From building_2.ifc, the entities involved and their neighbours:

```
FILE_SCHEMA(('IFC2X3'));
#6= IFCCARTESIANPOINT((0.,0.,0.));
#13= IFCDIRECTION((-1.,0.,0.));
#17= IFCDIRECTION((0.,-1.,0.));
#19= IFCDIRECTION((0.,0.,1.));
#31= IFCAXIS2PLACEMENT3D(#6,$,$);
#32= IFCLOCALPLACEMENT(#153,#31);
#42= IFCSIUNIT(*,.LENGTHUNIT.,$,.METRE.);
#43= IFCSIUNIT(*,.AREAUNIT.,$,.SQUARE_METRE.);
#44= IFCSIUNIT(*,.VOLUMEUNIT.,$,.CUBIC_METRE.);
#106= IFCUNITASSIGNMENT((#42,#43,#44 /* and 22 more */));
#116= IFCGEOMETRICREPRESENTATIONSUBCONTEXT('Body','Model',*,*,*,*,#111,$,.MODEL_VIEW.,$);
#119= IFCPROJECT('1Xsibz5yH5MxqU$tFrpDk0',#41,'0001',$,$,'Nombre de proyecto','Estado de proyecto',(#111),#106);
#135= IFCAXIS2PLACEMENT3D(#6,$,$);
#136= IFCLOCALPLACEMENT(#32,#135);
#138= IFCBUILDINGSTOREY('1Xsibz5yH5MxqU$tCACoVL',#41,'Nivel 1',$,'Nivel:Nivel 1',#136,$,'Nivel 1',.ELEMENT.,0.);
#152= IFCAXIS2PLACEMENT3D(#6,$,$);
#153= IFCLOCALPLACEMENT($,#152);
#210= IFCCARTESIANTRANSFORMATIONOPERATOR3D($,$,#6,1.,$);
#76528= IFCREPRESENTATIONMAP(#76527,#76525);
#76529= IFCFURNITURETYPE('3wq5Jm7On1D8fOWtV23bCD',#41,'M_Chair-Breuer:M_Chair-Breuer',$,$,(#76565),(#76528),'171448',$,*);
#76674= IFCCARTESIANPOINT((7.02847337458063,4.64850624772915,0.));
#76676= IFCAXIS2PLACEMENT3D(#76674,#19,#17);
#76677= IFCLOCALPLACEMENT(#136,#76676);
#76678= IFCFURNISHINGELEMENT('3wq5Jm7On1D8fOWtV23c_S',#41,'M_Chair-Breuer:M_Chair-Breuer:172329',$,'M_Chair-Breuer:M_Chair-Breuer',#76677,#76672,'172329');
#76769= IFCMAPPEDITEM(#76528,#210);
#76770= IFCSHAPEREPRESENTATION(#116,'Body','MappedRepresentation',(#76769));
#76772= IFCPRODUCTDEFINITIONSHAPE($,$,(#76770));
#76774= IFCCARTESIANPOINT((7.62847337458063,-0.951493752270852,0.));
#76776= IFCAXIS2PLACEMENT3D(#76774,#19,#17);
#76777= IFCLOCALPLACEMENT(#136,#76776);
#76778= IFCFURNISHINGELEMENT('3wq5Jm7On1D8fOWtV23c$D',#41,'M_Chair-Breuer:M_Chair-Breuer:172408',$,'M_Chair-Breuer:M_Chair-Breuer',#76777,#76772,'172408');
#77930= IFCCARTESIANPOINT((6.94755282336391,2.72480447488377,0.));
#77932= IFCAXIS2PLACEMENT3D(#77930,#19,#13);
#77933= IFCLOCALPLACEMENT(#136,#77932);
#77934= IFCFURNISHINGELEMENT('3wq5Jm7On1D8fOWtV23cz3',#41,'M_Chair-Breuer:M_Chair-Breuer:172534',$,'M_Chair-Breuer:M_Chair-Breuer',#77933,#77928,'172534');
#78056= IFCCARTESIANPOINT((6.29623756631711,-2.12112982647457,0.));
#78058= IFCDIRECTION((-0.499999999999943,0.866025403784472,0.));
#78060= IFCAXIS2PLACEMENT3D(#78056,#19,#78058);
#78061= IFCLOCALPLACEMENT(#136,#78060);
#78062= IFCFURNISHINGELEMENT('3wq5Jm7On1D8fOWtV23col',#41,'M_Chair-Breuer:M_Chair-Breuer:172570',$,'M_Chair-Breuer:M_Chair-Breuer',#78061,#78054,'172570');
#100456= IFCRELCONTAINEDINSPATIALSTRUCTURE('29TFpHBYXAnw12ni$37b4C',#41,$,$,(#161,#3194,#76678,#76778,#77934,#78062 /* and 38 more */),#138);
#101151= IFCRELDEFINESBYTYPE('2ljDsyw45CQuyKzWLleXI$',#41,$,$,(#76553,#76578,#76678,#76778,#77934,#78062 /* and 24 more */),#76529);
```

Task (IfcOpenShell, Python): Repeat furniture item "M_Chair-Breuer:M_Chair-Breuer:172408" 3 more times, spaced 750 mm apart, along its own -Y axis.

```python
import ifcopenshell
import ifcopenshell.api.geometry
import ifcopenshell.api.root
import ifcopenshell.util.element
import ifcopenshell.util.placement
import ifcopenshell.util.unit

model = ifcopenshell.open("building_2.ifc")
unit_scale = ifcopenshell.util.unit.calculate_unit_scale(model)


def reuse_history(source, copy):
    """copy_class also copies each property set's owner history, people and application; keep the originals."""
    for rel in copy.IsDefinedBy:
        if rel.is_a("IfcRelDefinesByProperties") and (history := rel.RelatingPropertyDefinition.OwnerHistory):
            rel.RelatingPropertyDefinition.OwnerHistory = source.OwnerHistory
            ifcopenshell.util.element.remove_deep2(model, history)


source = model.by_guid("3wq5Jm7On1D8fOWtV23c$D")
base = ifcopenshell.util.placement.get_local_placement(source.ObjectPlacement)
step = -base[:3, 1] * 0.75 / unit_scale

for i in range(1, 4):
    copy = ifcopenshell.api.root.copy_class(model, product=source)
    copy.Representation = ifcopenshell.util.element.copy_deep(
        model, source.Representation, exclude=["IfcGeometricRepresentationContext", "IfcRepresentationMap"]
    )
    copy.Name = "M_Chair-Breuer:M_Chair-Breuer"
    copy.Tag = None
    reuse_history(source, copy)
    matrix = base.copy()
    matrix[:3, 3] += i * step
    print("added at", matrix[:3, 3].round(3) + 0.0)
    ifcopenshell.api.geometry.edit_object_placement(model, product=copy, matrix=matrix, is_si=False)

model.write("building_2_v2.ifc")
```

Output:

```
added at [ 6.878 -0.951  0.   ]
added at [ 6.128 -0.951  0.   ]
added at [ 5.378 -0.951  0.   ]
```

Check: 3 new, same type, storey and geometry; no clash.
